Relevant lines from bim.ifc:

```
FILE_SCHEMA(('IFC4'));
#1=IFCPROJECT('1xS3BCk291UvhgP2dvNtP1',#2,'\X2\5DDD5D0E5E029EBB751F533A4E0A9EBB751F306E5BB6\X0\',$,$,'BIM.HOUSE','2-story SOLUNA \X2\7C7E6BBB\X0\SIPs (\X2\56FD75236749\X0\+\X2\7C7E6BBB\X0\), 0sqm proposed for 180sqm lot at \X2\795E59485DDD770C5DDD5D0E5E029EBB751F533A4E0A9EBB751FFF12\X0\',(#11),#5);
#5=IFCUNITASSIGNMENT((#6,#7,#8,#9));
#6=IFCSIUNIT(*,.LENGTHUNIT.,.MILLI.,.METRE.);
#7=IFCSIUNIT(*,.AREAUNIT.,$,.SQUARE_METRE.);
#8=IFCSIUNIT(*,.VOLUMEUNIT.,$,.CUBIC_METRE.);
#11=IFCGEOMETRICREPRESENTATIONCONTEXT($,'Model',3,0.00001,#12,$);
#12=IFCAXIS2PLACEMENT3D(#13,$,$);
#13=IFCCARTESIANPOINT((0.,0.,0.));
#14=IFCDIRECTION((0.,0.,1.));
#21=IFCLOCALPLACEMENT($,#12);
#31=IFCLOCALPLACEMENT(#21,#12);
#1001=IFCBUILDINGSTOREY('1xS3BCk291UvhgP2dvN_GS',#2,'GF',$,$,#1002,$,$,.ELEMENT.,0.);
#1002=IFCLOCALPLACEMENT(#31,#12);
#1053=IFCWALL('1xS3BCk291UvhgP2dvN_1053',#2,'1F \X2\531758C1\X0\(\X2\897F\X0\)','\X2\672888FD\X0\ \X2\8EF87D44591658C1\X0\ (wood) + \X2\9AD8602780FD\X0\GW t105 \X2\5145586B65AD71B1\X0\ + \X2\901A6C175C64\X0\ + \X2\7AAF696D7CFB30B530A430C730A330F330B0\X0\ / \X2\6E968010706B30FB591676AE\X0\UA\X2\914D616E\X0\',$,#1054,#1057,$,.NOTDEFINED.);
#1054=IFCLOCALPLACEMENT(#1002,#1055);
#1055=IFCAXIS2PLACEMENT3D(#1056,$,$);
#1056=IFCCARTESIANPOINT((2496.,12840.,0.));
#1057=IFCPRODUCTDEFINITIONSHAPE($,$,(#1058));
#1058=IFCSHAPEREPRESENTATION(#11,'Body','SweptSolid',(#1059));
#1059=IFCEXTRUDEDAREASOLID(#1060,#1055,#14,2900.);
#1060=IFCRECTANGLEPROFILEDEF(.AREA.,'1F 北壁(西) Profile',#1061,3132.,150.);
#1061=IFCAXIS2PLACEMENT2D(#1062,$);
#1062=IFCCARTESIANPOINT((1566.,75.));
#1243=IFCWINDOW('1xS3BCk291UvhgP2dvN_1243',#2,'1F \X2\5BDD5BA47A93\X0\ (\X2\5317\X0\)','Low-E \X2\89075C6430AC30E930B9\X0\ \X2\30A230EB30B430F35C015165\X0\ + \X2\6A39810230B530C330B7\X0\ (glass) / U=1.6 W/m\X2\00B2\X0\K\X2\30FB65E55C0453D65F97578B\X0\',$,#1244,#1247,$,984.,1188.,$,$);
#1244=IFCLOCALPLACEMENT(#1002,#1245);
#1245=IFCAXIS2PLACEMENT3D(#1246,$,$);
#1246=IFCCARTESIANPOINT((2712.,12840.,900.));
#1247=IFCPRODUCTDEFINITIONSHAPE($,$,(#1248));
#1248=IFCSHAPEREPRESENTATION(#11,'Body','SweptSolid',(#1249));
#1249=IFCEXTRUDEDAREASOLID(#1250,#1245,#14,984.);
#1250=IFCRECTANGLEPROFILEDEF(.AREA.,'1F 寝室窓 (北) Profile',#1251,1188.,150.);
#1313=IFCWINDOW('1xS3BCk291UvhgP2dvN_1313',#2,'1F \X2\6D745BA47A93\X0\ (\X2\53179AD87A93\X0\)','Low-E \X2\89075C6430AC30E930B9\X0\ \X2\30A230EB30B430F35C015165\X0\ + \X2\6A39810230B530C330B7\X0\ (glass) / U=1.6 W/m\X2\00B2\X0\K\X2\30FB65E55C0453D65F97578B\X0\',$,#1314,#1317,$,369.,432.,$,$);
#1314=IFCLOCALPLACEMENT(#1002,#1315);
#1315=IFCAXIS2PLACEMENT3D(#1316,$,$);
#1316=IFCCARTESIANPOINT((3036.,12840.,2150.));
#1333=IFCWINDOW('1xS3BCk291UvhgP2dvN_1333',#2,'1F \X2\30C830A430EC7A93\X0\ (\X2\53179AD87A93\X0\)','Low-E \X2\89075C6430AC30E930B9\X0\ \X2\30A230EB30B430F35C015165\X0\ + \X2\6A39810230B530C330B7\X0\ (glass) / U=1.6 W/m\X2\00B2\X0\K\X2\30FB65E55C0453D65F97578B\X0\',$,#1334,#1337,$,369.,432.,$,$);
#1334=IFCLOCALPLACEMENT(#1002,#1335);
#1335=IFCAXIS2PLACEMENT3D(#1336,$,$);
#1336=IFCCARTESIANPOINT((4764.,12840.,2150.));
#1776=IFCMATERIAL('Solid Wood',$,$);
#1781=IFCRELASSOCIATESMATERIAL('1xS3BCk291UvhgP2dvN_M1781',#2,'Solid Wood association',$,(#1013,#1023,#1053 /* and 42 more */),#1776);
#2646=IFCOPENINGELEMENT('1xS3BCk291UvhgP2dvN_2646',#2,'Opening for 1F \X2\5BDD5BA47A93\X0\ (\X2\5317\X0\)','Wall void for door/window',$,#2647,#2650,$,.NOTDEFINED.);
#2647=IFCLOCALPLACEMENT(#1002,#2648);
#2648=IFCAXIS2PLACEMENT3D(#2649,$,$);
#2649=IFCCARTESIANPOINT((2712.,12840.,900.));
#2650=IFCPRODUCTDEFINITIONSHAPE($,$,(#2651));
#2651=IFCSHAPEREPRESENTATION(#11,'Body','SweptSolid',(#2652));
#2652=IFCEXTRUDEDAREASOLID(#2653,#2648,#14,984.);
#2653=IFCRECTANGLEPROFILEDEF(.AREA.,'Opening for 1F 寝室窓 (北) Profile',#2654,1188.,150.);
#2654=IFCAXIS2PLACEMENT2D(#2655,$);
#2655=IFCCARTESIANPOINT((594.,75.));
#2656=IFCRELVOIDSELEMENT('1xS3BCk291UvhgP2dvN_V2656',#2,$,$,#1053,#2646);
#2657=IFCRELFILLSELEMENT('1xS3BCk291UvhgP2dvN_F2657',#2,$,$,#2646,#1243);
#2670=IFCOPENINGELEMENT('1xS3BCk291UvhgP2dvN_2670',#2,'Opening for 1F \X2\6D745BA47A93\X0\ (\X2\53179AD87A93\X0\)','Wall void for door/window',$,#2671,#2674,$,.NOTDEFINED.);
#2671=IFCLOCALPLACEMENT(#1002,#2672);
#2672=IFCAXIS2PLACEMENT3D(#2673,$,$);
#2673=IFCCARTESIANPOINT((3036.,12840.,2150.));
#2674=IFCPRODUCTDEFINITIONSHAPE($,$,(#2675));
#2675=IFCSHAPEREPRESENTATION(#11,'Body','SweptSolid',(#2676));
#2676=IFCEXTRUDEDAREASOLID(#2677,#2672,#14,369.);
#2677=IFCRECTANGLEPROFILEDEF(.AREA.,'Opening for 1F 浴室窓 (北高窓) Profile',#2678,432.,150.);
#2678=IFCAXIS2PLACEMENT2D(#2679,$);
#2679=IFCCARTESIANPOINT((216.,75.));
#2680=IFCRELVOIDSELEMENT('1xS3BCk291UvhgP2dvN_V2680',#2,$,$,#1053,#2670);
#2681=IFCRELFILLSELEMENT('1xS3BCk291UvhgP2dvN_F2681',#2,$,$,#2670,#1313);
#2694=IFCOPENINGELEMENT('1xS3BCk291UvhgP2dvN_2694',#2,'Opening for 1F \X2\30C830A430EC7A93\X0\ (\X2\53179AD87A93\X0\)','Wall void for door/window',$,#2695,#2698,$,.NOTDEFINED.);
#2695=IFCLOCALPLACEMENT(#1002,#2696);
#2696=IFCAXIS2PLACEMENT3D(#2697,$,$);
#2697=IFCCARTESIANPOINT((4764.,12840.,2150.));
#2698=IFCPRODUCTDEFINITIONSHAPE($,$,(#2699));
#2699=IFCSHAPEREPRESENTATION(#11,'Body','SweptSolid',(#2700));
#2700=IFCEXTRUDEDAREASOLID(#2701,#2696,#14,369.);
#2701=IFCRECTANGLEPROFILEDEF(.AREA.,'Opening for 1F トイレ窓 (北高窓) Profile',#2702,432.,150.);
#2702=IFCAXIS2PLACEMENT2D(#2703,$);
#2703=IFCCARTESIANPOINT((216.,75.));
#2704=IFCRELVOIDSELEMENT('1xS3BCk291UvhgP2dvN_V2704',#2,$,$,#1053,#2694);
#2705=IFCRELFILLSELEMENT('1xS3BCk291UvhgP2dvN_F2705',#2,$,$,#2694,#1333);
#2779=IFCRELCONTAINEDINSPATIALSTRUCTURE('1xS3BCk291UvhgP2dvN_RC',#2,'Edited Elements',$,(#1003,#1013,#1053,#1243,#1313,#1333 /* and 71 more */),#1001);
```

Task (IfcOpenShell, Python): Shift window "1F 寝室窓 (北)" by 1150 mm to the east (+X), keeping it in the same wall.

```python
import ifcopenshell
import ifcopenshell.api.geometry
import ifcopenshell.util.placement

model = ifcopenshell.open("bim.ifc")

window = model.by_id(1243)
opening = window.FillsVoids[0].RelatingOpeningElement
wall = opening.VoidsElements[0].RelatingBuildingElement

wall_matrix = ifcopenshell.util.placement.get_local_placement(wall.ObjectPlacement)
shift = wall_matrix[:3, 0] * 1150.0
before = ifcopenshell.util.placement.get_local_placement(window.ObjectPlacement)[:3, 3].copy()

# The window is not placed relative to its opening, so move both.
for product in (opening, window):
    matrix = ifcopenshell.util.placement.get_local_placement(product.ObjectPlacement)
    matrix[:3, 3] += shift
    ifcopenshell.api.geometry.edit_object_placement(model, product=product, matrix=matrix, is_si=False)

after = ifcopenshell.util.placement.get_local_placement(window.ObjectPlacement)[:3, 3]
print("window moved by", (after - before).round(3) + 0.0)

model.write("bim-out.ifc")
```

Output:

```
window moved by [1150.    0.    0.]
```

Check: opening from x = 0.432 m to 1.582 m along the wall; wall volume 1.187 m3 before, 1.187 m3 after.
